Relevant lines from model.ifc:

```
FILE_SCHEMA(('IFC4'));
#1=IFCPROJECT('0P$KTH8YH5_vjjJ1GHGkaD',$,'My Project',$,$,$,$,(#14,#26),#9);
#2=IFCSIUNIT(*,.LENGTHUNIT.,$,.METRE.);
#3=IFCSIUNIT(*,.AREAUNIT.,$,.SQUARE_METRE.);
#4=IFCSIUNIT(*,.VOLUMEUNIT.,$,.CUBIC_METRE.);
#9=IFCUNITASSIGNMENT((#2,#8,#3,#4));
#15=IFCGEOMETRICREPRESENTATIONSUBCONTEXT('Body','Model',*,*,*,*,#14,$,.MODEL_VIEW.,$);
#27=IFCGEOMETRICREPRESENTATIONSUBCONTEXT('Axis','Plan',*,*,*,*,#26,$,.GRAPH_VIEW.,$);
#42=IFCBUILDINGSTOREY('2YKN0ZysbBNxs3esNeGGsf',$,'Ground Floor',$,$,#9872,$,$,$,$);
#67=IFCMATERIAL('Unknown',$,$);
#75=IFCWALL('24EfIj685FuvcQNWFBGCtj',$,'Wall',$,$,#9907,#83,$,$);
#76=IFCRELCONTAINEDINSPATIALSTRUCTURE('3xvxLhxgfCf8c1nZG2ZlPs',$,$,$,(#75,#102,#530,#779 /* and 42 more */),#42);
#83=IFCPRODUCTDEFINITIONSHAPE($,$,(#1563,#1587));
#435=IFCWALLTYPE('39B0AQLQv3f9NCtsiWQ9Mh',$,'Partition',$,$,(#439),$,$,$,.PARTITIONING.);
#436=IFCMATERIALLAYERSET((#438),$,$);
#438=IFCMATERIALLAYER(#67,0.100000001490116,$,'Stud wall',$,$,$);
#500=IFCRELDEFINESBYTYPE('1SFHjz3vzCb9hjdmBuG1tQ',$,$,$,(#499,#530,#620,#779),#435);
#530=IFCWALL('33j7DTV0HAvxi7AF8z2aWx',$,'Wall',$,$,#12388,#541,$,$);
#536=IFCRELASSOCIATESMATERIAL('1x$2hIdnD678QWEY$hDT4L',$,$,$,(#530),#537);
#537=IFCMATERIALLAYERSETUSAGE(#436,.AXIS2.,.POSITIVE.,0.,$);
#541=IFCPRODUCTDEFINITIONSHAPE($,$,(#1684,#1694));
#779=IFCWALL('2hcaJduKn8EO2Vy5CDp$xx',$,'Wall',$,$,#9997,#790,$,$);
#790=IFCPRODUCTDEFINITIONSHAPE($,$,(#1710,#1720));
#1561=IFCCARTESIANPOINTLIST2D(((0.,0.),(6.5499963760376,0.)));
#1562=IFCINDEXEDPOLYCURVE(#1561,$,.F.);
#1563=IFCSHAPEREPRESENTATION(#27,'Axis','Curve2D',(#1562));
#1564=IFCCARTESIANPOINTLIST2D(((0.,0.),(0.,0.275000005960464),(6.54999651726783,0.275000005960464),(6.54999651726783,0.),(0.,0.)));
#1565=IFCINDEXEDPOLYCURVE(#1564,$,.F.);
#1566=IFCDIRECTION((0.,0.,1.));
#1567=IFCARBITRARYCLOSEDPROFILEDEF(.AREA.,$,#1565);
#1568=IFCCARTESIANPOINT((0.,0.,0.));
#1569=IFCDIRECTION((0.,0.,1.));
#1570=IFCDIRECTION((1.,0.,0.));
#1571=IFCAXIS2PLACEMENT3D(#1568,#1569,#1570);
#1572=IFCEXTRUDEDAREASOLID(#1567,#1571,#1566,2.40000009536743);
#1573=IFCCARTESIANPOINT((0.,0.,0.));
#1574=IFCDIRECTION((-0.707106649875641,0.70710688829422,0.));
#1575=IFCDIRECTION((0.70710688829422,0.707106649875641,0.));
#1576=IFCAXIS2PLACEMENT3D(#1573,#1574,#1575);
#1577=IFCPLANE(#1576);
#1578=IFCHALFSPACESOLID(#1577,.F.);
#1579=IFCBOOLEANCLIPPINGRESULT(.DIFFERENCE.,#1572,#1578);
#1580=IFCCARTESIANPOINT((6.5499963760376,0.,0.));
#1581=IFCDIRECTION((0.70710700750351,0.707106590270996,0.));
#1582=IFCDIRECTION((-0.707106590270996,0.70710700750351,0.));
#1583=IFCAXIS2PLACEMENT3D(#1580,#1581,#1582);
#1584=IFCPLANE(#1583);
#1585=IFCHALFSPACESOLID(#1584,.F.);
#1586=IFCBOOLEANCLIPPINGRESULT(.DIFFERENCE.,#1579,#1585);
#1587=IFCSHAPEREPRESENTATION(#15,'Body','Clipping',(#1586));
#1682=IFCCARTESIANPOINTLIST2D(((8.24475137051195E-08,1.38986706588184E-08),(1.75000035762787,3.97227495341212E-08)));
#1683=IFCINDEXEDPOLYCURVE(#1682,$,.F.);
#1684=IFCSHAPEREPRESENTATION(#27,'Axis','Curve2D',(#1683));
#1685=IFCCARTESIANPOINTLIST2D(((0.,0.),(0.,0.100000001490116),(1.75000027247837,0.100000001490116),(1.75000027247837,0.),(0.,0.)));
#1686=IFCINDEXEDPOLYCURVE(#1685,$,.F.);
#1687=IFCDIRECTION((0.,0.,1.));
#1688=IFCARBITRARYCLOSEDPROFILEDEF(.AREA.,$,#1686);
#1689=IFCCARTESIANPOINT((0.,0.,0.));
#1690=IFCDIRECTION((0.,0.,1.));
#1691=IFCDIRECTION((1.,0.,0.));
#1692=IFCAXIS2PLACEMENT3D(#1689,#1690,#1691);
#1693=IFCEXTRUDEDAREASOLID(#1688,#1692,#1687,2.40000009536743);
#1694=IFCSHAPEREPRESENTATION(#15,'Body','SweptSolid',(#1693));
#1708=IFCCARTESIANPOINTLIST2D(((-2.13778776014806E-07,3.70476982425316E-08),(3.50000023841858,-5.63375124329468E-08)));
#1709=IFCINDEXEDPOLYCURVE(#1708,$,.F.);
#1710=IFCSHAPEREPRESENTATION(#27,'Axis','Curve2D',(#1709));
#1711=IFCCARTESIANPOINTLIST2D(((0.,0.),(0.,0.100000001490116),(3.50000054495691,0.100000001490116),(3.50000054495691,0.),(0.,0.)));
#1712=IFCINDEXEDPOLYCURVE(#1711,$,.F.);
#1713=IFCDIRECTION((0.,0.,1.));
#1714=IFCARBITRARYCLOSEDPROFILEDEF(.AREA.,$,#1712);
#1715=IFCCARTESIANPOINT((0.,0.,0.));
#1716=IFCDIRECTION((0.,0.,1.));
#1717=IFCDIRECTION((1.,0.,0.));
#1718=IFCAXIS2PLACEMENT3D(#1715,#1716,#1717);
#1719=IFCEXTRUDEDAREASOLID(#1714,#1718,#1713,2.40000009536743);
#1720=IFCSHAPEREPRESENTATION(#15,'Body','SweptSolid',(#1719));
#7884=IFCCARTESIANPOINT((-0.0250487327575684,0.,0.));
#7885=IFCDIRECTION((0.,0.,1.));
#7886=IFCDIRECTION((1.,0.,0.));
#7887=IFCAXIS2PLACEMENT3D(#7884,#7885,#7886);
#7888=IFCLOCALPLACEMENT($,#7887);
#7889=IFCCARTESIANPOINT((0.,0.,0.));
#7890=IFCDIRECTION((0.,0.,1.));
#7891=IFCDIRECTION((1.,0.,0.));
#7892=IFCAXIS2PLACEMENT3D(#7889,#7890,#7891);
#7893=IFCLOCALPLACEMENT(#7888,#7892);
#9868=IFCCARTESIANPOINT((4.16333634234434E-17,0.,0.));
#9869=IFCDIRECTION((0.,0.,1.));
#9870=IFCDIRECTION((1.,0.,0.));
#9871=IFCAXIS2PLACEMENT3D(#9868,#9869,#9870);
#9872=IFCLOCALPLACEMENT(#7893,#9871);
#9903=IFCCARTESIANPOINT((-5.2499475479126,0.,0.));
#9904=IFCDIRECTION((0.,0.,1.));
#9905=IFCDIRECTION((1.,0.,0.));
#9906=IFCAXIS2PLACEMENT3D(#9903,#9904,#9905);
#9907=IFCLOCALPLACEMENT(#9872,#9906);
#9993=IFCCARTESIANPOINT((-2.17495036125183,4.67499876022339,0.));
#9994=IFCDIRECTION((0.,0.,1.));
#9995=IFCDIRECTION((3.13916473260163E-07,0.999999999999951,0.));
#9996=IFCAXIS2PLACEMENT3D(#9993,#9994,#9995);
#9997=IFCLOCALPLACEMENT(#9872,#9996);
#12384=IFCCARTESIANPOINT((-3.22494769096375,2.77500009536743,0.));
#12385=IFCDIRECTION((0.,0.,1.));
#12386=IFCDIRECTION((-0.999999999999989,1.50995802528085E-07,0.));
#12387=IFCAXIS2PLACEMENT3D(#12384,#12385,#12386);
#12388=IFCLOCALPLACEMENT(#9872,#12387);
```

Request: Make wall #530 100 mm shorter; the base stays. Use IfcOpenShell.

```python
import ifcopenshell
import ifcopenshell.geom
import ifcopenshell.util.representation
import ifcopenshell.util.shape

model = ifcopenshell.open("model.ifc")
settings = ifcopenshell.geom.settings()


def volume(element):
    """Net volume in cubic metres, openings subtracted."""
    shape = ifcopenshell.geom.create_shape(settings, element)
    return ifcopenshell.util.shape.get_volume(shape.geometry)


wall = model.by_guid("33j7DTV0HAvxi7AF8z2aWx")
before = volume(wall)

body = ifcopenshell.util.representation.get_representation(wall, "Model", "Body")
solid = body.Items[0]
old_height = solid.Depth
solid.Depth -= 0.1
after = volume(wall)

print(f"height {old_height:g} -> {solid.Depth:g}, volume {before:.3f} -> {after:.3f} m3")

model.write("model_edited.ifc")
```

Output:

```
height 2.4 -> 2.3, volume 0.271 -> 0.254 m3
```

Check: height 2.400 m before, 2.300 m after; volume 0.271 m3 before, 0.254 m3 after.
